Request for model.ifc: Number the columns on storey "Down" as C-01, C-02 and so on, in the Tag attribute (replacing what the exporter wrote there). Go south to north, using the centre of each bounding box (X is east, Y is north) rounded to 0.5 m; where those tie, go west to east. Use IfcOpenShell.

First a look at what the model holds.

```python
import ifcopenshell
import ifcopenshell.util.element
import ifcopenshell.util.placement

model = ifcopenshell.open("model.ifc")
print(model.schema)
storey = next(s for s in model.by_type("IfcBuildingStorey") if s.Name == "Down")
columns = [e for e in ifcopenshell.util.element.get_decomposition(storey) if e.is_a("IfcColumn")]
for e in sorted(columns, key=lambda e: e.id()):
    origin = ifcopenshell.util.placement.get_local_placement(e.ObjectPlacement)[:3, 3]
    print(e.id(), e.Tag, e.Name, origin.round(2) + 0.0, sep=" | ")
```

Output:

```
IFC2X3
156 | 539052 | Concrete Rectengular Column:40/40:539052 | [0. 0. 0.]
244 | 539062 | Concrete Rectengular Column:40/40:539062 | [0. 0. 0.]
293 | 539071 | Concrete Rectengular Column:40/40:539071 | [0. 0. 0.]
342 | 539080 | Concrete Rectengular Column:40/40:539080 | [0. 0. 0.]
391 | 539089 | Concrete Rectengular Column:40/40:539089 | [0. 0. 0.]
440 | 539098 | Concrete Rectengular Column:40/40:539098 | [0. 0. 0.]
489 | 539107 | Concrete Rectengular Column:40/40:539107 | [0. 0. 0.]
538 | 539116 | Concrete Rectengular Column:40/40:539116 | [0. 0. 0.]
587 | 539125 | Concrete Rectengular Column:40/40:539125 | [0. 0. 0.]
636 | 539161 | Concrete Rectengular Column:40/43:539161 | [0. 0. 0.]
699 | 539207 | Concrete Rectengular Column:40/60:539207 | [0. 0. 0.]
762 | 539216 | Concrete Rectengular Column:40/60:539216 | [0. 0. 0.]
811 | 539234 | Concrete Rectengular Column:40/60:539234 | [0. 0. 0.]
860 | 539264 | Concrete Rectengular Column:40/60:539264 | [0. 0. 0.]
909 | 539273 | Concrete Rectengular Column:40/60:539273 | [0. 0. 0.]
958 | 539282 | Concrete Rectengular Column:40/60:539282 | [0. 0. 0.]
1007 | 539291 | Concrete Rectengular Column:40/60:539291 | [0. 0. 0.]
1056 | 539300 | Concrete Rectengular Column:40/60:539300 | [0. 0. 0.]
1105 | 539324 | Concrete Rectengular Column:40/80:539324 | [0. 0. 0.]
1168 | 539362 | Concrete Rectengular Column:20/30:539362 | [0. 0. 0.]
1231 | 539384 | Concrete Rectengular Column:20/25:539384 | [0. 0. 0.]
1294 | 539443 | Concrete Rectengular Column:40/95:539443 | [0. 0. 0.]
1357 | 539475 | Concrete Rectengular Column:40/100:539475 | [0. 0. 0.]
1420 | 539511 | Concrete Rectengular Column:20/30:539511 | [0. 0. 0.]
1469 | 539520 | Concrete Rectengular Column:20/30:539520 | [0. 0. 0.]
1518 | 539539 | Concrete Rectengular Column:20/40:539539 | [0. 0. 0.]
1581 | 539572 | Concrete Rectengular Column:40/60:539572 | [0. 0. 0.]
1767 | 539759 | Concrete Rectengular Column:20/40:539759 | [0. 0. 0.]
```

```python
import ifcopenshell
import ifcopenshell.geom
import ifcopenshell.util.element
import ifcopenshell.util.shape

model = ifcopenshell.open("model.ifc")
settings = ifcopenshell.geom.settings()
settings.set("use-world-coords", True)


def centre(element):
    shape = ifcopenshell.geom.create_shape(settings, element)
    return ifcopenshell.util.shape.get_bbox_centroid(shape.geometry)


storey = next(s for s in model.by_type("IfcBuildingStorey") if s.Name == "Down")
columns = [e for e in ifcopenshell.util.element.get_decomposition(storey) if e.is_a("IfcColumn")]

# Insertion points can sit at a corner or the storey origin, so sort by the geometry (in metres).
centres = {e: centre(e) for e in columns}
columns.sort(key=lambda e: (round(centres[e][1] / 0.5), centres[e][0]))

for i, e in enumerate(columns, start=1):
    number = f"C-{i:02d}"
    e.Tag = number
    print(e.id(), number)

model.write("model_v2.ifc")
```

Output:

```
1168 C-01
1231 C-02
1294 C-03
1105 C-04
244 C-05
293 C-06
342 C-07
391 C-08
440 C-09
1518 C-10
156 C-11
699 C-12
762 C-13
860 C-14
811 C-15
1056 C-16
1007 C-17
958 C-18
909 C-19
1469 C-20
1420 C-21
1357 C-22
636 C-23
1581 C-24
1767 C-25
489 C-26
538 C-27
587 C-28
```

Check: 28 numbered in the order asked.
